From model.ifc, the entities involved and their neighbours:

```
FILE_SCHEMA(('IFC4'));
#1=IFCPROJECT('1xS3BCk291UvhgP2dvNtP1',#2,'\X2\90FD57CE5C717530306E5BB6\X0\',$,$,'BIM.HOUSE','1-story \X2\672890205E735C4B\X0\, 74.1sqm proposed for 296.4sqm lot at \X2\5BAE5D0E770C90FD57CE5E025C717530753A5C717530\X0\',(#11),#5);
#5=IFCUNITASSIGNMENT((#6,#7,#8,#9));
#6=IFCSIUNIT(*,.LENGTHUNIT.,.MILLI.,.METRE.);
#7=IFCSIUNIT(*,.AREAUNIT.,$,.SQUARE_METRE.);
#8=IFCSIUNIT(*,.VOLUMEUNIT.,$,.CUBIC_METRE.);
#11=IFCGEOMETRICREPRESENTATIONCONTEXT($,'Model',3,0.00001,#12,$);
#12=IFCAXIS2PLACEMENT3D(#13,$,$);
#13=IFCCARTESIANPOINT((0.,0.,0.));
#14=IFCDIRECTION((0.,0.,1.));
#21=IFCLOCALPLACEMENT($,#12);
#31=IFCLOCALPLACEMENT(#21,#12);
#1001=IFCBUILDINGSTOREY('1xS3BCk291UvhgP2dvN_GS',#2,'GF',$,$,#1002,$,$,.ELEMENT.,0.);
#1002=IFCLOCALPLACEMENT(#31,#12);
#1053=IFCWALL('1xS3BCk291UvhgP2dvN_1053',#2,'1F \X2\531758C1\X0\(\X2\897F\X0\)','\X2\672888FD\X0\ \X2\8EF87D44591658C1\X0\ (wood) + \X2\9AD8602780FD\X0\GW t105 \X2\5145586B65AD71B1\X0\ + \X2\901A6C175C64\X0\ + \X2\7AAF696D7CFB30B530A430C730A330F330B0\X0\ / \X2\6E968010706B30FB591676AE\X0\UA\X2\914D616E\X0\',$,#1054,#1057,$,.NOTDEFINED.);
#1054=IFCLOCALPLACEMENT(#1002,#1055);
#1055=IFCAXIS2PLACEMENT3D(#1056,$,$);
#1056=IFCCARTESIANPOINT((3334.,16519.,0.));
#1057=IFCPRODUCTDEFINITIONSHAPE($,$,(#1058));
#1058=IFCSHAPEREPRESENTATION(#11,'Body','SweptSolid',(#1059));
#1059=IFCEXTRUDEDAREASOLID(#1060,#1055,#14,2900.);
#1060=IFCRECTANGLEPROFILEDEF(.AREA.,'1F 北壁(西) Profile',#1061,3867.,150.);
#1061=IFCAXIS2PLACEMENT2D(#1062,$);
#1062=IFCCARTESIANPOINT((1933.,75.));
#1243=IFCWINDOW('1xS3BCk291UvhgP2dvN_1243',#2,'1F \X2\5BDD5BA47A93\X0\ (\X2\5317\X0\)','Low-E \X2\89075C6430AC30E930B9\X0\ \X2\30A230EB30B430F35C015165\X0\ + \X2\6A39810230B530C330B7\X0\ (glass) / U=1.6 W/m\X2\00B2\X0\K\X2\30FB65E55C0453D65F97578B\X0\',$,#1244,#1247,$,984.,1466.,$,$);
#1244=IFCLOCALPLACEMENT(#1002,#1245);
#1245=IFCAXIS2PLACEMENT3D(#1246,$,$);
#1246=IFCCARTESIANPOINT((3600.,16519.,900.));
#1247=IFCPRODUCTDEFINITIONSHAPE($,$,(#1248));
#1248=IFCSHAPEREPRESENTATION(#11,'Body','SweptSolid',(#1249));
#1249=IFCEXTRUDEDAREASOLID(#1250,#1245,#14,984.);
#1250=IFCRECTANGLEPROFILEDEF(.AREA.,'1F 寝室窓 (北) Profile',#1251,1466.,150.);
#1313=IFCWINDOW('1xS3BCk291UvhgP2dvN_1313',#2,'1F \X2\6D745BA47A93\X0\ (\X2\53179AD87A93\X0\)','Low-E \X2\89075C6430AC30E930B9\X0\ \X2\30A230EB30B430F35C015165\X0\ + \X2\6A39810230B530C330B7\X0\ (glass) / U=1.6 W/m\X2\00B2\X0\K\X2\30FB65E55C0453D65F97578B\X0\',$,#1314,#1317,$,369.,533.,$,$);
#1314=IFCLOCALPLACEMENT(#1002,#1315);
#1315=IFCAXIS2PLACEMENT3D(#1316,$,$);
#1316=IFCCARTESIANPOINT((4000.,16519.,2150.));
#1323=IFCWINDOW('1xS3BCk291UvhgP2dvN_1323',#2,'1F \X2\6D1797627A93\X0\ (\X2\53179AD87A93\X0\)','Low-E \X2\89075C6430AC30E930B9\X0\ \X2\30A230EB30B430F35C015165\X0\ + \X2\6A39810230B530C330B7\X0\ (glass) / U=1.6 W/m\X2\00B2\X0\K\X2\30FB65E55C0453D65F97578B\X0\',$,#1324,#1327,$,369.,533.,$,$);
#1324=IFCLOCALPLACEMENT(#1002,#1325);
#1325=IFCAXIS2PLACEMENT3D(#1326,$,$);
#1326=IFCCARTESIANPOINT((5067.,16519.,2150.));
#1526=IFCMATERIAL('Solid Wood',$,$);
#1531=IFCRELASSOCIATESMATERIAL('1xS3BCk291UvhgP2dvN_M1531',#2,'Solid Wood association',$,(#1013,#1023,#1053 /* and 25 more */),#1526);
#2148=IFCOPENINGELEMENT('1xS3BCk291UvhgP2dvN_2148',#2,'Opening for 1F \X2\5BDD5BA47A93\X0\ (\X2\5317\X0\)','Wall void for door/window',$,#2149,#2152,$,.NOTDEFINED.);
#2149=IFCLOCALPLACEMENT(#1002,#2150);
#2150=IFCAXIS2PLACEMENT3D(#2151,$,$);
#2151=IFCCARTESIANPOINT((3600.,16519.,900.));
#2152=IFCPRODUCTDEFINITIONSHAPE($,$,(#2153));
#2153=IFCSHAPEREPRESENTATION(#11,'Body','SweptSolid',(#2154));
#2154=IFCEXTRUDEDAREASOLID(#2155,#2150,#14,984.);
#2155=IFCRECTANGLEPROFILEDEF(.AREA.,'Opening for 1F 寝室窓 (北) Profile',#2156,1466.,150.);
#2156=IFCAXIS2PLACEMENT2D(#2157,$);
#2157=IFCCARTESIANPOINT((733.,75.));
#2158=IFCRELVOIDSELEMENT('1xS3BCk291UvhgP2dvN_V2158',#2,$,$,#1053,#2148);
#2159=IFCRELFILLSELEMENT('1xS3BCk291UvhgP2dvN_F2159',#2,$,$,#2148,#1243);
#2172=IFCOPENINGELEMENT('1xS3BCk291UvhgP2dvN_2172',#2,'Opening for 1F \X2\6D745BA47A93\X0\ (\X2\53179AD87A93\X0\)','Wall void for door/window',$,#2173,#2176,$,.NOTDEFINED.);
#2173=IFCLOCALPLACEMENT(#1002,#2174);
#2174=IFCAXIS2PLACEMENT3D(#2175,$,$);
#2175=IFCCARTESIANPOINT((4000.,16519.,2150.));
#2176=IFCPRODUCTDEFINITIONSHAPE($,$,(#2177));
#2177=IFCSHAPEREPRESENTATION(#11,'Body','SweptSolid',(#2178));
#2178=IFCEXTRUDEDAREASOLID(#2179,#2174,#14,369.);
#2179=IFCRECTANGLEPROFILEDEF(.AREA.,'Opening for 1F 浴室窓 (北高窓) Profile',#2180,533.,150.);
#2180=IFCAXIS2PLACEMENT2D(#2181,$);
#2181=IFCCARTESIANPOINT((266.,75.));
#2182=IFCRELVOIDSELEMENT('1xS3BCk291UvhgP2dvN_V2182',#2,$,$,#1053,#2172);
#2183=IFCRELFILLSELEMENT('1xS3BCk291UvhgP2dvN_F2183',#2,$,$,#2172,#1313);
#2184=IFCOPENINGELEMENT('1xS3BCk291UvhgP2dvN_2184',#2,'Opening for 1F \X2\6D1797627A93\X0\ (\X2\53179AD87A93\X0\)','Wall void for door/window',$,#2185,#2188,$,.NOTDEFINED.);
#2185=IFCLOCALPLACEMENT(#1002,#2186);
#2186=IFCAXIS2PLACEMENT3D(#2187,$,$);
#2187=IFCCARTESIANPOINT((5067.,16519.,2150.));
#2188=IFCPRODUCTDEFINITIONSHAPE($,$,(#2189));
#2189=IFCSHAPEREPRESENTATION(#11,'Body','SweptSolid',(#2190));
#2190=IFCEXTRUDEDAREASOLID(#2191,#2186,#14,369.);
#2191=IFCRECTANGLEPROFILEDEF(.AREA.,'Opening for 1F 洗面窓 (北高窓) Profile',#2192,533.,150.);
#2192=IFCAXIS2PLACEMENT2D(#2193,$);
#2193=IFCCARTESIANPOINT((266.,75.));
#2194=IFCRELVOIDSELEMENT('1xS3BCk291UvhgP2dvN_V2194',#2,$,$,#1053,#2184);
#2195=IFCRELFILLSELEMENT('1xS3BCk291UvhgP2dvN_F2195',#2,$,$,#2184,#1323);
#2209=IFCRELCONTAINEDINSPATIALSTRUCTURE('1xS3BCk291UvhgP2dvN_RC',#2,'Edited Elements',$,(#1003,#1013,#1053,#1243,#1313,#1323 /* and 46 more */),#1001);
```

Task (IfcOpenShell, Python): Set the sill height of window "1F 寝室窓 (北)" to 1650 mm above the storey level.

```python
import numpy as np
import ifcopenshell
import ifcopenshell.api.geometry
import ifcopenshell.geom
import ifcopenshell.util.element
import ifcopenshell.util.placement
import ifcopenshell.util.shape
import ifcopenshell.util.unit

model = ifcopenshell.open("model.ifc")
unit_scale = ifcopenshell.util.unit.calculate_unit_scale(model)

window = model.by_guid("1xS3BCk291UvhgP2dvN_1243")
opening = window.FillsVoids[0].RelatingOpeningElement
storey = ifcopenshell.util.element.get_container(window, ifc_class="IfcBuildingStorey")
level = ifcopenshell.util.placement.get_local_placement(storey.ObjectPlacement)[2, 3]

# The opening's origin need not be at the sill, so measure its lowest point.
shape = ifcopenshell.geom.create_shape(ifcopenshell.geom.settings(), opening)
bottom = ifcopenshell.util.shape.get_shape_bottom_elevation(shape, shape.geometry) / unit_scale
dz = level + 1.65 / unit_scale - bottom

shift = np.array([0.0, 0.0, dz])
# The window is not placed relative to its opening, so move both.
for product in (opening, window):
    matrix = ifcopenshell.util.placement.get_local_placement(product.ObjectPlacement)
    matrix[:3, 3] += shift
    ifcopenshell.api.geometry.edit_object_placement(model, product=product, matrix=matrix, is_si=False)

print(f"moved by {dz * unit_scale:+.3f} m")

model.write("model_rev.ifc")
```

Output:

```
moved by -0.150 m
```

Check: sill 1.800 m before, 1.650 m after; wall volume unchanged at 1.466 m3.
